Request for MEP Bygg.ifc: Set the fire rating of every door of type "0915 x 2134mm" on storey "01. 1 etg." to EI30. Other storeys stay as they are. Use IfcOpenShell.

First a look at what the model holds.

```python
import ifcopenshell
import ifcopenshell.util.element

model = ifcopenshell.open("MEP Bygg.ifc")
print(model.schema)
storey = next(s for s in model.by_type("IfcBuildingStorey") if s.Name == "01. 1 etg.")
doors = [e for e in ifcopenshell.util.element.get_decomposition(storey) if e.is_a("IfcDoor")]
seen = {}
for e in doors:
    element_type = ifcopenshell.util.element.get_type(e)
    key = (element_type.Name if element_type != e and element_type else None, ifcopenshell.util.element.get_pset(e, "Pset_DoorCommon", "FireRating"))
    seen[key] = seen.get(key, 0) + 1
for (name, value), count in sorted(seen.items(), key=str):
    print(count, "x", name, "|", value)
```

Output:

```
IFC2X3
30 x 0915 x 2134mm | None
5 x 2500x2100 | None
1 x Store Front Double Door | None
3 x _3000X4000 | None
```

```python
import ifcopenshell
import ifcopenshell.api.pset
import ifcopenshell.util.element

model = ifcopenshell.open("MEP Bygg.ifc")

storey = next(s for s in model.by_type("IfcBuildingStorey") if s.Name == "01. 1 etg.")
doors = [e for e in ifcopenshell.util.element.get_decomposition(storey) if e.is_a("IfcDoor")]

count = 0
for e in doors:
    element_type = ifcopenshell.util.element.get_type(e)
    if element_type in (None, e) or element_type.Name != "0915 x 2134mm":
        continue
    # add_pset returns the element's existing set when there is one.
    pset = ifcopenshell.api.pset.add_pset(model, product=e, name="Pset_DoorCommon")
    ifcopenshell.api.pset.edit_pset(model, pset=pset, properties={"FireRating": "EI30"})
    count += 1

print(count, "doors updated")

model.write("MEP Bygg_edited.ifc")
```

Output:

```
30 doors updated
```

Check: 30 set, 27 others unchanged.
